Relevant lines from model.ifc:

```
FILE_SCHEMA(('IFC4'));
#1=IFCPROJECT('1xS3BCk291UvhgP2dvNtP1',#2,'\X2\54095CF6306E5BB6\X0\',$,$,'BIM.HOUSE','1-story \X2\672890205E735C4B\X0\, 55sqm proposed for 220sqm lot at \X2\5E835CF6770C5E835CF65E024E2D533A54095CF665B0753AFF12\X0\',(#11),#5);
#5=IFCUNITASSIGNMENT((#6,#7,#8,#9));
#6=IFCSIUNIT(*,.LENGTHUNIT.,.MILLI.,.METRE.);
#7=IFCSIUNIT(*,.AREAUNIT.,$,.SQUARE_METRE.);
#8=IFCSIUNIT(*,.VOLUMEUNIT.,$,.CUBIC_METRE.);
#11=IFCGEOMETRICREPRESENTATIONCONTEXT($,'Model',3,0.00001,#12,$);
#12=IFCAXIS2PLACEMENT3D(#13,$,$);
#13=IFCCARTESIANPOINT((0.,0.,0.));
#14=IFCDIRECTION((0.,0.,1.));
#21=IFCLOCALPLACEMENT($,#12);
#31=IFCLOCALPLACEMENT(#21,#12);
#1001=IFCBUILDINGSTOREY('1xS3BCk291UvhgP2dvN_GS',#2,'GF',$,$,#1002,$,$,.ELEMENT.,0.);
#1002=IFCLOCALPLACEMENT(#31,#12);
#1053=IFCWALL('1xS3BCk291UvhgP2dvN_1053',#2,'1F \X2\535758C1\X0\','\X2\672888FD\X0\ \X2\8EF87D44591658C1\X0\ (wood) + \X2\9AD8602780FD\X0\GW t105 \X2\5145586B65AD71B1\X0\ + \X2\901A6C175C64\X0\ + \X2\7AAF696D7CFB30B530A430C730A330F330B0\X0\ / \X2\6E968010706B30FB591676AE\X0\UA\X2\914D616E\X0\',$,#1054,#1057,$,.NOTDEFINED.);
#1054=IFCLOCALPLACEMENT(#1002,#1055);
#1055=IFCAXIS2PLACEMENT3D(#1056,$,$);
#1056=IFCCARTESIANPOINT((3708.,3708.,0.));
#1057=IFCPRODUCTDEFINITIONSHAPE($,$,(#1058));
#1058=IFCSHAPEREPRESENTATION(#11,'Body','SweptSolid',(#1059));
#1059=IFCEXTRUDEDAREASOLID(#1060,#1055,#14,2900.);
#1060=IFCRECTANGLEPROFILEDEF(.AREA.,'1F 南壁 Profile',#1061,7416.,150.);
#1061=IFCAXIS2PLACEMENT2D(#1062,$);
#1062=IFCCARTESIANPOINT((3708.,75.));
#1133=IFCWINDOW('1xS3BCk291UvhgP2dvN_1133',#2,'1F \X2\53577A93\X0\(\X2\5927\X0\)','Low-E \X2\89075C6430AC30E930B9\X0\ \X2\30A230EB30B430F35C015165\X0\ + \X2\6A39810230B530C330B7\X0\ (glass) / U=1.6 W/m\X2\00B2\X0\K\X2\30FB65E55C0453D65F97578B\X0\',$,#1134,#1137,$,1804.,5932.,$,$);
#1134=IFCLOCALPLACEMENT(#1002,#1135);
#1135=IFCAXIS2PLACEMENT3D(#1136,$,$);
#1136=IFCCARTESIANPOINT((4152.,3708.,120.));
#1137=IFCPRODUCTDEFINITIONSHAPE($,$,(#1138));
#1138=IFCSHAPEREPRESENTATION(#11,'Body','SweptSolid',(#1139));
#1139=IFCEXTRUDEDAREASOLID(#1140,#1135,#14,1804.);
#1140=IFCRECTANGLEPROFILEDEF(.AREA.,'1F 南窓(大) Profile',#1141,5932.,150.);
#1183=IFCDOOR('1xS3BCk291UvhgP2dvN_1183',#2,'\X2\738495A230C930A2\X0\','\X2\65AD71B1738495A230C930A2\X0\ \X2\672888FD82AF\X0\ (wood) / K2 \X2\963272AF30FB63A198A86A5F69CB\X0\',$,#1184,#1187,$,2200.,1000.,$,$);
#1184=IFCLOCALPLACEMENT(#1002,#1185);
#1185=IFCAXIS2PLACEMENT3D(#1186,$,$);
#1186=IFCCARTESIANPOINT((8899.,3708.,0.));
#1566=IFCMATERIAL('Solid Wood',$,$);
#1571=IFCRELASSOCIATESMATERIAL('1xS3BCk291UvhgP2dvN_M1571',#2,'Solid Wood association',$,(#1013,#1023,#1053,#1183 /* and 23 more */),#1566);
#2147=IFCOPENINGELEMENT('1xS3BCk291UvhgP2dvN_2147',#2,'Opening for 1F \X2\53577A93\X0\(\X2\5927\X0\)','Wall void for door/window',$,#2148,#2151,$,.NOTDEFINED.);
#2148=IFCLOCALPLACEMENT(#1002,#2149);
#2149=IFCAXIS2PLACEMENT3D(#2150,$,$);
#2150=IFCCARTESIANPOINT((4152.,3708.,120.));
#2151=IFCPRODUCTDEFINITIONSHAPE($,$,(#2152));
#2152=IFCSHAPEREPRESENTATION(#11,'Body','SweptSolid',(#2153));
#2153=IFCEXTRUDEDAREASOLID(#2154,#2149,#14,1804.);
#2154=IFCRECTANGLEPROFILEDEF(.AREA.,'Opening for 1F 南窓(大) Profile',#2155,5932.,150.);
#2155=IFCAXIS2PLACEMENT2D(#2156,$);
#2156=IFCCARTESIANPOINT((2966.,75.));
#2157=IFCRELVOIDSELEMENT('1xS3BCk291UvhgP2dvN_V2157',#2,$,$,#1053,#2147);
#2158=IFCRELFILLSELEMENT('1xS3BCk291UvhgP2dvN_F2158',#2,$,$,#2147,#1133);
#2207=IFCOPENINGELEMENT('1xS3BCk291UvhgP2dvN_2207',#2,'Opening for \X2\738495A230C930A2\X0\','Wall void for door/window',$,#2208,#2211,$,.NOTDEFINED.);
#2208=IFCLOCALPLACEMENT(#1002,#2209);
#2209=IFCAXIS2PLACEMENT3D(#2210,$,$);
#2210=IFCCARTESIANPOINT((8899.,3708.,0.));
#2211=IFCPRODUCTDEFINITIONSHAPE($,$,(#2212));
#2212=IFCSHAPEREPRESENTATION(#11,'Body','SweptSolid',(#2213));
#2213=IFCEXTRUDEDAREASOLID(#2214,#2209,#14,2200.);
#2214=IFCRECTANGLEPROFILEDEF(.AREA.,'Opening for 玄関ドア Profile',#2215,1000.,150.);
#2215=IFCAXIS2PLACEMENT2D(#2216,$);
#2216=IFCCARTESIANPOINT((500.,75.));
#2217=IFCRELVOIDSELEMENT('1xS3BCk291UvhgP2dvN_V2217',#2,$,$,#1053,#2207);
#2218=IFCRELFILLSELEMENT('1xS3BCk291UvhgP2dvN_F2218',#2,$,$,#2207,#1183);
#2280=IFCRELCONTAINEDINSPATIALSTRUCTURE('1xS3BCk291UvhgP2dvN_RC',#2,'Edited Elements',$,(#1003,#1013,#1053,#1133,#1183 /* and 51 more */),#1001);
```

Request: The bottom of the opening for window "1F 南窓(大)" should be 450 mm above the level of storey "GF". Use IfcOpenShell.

```python
import numpy as np
import ifcopenshell
import ifcopenshell.api.geometry
import ifcopenshell.geom
import ifcopenshell.util.element
import ifcopenshell.util.placement
import ifcopenshell.util.shape
import ifcopenshell.util.unit

model = ifcopenshell.open("model.ifc")
unit_scale = ifcopenshell.util.unit.calculate_unit_scale(model)

window = model.by_id(1133)
opening = window.FillsVoids[0].RelatingOpeningElement
storey = ifcopenshell.util.element.get_container(window, ifc_class="IfcBuildingStorey")
level = ifcopenshell.util.placement.get_local_placement(storey.ObjectPlacement)[2, 3]

# The opening's origin need not be at the sill, so measure its lowest point.
shape = ifcopenshell.geom.create_shape(ifcopenshell.geom.settings(), opening)
bottom = ifcopenshell.util.shape.get_shape_bottom_elevation(shape, shape.geometry) / unit_scale
dz = level + 450.0 - bottom

shift = np.array([0.0, 0.0, dz])
# The window is not placed relative to its opening, so move both.
for product in (opening, window):
    matrix = ifcopenshell.util.placement.get_local_placement(product.ObjectPlacement)
    matrix[:3, 3] += shift
    ifcopenshell.api.geometry.edit_object_placement(model, product=product, matrix=matrix, is_si=False)

print(f"moved by {dz * unit_scale:+.3f} m")

model.write("model_updated.ifc")
```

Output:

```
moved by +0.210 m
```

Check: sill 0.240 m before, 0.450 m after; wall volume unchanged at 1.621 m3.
